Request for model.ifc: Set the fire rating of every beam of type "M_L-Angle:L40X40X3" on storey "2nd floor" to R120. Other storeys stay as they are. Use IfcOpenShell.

First a look at what the model holds.

```python
import ifcopenshell
import ifcopenshell.util.element

model = ifcopenshell.open("model.ifc")
print(model.schema)
storey = next(s for s in model.by_type("IfcBuildingStorey") if s.Name == "2nd floor")
beams = [e for e in ifcopenshell.util.element.get_decomposition(storey) if e.is_a("IfcBeam")]
seen = {}
for e in beams:
    element_type = ifcopenshell.util.element.get_type(e)
    key = (element_type.Name if element_type != e and element_type else None, ifcopenshell.util.element.get_pset(e, "Pset_BeamCommon", "FireRating"))
    seen[key] = seen.get(key, 0) + 1
for (name, value), count in sorted(seen.items(), key=str):
    print(count, "x", name, "|", value)
```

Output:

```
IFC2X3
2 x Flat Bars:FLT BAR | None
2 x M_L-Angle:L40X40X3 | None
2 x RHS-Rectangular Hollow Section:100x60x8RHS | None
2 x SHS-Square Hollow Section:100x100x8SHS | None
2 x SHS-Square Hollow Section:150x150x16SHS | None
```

```python
import ifcopenshell
import ifcopenshell.api.pset
import ifcopenshell.util.element

model = ifcopenshell.open("model.ifc")

storey = next(s for s in model.by_type("IfcBuildingStorey") if s.Name == "2nd floor")
beams = [e for e in ifcopenshell.util.element.get_decomposition(storey) if e.is_a("IfcBeam")]

count = 0
for e in beams:
    element_type = ifcopenshell.util.element.get_type(e)
    if element_type in (None, e) or element_type.Name != "M_L-Angle:L40X40X3":
        continue
    # add_pset returns the element's existing set when there is one.
    pset = ifcopenshell.api.pset.add_pset(model, product=e, name="Pset_BeamCommon")
    ifcopenshell.api.pset.edit_pset(model, pset=pset, properties={"FireRating": "R120"})
    count += 1

print(count, "beams updated")

model.write("model_edited.ifc")
```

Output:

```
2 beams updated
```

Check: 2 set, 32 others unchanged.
